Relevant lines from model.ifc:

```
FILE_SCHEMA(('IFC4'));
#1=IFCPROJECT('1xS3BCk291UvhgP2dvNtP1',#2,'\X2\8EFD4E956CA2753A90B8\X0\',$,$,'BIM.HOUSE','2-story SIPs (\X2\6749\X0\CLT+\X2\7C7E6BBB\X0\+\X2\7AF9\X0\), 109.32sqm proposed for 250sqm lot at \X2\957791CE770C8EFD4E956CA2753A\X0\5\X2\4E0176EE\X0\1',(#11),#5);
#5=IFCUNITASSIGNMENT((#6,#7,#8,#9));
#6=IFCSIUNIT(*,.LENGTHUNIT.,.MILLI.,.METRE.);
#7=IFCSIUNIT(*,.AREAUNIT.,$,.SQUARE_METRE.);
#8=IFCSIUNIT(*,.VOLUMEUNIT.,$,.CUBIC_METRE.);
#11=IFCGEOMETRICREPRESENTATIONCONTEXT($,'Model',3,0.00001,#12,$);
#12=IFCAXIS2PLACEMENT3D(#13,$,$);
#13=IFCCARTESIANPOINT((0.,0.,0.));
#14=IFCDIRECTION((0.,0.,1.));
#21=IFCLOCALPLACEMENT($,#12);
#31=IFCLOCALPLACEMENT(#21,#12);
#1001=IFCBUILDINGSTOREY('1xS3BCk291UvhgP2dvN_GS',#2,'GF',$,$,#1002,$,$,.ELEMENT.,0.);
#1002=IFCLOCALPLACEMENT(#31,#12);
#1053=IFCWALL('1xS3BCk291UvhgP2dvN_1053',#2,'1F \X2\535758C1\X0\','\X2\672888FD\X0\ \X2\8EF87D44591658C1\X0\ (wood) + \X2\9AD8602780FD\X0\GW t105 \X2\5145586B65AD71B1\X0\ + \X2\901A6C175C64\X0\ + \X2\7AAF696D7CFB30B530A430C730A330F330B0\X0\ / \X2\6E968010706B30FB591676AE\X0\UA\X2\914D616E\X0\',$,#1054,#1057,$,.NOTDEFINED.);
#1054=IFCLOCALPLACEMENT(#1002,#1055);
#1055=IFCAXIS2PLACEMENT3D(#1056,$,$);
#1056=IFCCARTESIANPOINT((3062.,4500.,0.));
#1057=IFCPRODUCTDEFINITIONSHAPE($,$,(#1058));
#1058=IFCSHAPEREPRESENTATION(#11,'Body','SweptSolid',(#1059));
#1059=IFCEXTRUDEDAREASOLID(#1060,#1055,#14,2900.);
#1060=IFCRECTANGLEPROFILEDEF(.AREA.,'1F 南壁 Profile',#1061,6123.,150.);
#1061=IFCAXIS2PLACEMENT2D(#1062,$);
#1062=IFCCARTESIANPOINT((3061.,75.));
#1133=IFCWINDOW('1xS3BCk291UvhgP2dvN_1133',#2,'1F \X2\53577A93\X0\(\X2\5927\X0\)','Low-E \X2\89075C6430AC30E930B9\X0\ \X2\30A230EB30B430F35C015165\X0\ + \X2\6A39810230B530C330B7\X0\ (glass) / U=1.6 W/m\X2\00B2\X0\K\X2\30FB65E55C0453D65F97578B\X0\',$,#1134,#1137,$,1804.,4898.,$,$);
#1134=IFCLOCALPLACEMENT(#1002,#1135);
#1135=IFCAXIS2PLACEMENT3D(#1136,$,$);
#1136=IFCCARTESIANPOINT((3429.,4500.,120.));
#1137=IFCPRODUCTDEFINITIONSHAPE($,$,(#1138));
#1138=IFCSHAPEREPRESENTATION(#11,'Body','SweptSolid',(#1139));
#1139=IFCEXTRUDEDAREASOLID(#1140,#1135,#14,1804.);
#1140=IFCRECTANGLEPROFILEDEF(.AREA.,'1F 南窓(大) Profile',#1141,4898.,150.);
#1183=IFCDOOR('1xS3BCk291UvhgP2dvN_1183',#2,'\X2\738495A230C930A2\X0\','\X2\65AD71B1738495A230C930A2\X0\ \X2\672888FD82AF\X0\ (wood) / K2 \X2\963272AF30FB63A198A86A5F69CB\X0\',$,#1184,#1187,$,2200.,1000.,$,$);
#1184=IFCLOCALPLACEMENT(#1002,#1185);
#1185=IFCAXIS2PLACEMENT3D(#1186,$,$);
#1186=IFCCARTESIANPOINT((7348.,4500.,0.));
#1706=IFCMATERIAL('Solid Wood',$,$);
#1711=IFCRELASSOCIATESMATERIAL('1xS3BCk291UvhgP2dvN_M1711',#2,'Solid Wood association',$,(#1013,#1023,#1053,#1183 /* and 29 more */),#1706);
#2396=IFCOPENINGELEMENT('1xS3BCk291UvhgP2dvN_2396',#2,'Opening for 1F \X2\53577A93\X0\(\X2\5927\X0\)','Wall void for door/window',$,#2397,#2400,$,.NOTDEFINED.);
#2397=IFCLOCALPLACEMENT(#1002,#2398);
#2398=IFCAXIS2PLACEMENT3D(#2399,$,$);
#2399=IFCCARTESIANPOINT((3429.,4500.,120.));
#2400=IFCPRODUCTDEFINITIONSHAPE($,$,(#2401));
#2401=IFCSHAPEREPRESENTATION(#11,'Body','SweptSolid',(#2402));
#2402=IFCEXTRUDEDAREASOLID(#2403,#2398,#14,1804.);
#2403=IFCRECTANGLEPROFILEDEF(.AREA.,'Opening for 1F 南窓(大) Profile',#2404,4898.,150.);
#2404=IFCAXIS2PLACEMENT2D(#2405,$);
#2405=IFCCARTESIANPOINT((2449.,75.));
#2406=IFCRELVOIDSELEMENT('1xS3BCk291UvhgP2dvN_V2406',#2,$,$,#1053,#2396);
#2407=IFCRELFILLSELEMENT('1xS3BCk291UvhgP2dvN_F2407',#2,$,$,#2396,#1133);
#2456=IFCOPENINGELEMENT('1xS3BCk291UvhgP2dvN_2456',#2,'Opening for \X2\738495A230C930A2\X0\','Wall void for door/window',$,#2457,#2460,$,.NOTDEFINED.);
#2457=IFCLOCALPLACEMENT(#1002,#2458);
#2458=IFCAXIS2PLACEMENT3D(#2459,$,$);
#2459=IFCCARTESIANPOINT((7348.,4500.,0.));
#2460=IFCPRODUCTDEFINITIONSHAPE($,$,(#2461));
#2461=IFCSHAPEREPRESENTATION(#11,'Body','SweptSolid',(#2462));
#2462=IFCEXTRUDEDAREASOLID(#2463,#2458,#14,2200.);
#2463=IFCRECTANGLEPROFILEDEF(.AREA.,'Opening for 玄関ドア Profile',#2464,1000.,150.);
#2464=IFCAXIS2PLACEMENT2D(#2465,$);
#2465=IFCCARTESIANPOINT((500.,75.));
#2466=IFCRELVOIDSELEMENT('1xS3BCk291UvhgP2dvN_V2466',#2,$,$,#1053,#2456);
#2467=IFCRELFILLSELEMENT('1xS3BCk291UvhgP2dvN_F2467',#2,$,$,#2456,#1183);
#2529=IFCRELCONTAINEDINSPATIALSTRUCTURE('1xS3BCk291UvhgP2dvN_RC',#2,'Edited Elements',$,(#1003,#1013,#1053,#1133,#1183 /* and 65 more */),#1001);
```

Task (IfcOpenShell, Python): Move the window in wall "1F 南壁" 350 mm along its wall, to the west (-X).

```python
import ifcopenshell
import ifcopenshell.api.geometry
import ifcopenshell.util.placement
import ifcopenshell.util.unit

model = ifcopenshell.open("model.ifc")
unit_scale = ifcopenshell.util.unit.calculate_unit_scale(model)

window = model.by_guid("1xS3BCk291UvhgP2dvN_1133")
opening = window.FillsVoids[0].RelatingOpeningElement
wall = opening.VoidsElements[0].RelatingBuildingElement

wall_matrix = ifcopenshell.util.placement.get_local_placement(wall.ObjectPlacement)
shift = wall_matrix[:3, 0] * -0.35 / unit_scale
before = ifcopenshell.util.placement.get_local_placement(window.ObjectPlacement)[:3, 3].copy()

# The window is not placed relative to its opening, so move both.
for product in (opening, window):
    matrix = ifcopenshell.util.placement.get_local_placement(product.ObjectPlacement)
    matrix[:3, 3] += shift
    ifcopenshell.api.geometry.edit_object_placement(model, product=product, matrix=matrix, is_si=False)

after = ifcopenshell.util.placement.get_local_placement(window.ObjectPlacement)[:3, 3]
print("window moved by", (after - before).round(3) + 0.0)

model.write("model_rev.ifc")
```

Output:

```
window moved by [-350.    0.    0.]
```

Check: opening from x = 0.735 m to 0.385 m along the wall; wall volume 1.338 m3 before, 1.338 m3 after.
